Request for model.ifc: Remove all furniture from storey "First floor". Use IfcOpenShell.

First a look at what the model holds.

```python
import ifcopenshell
import ifcopenshell.util.element

model = ifcopenshell.open("model.ifc")
print(model.schema)
storey = next(s for s in model.by_type("IfcBuildingStorey") if s.Name == "First floor")
furniture = [e for e in ifcopenshell.util.element.get_decomposition(storey) if e.is_a("IfcFurnishingElement")]
seen = {}
for e in furniture:
    element_type = ifcopenshell.util.element.get_type(e)
    name = element_type.Name if element_type not in (None, e) else None
    seen[name] = seen.get(name, 0) + 1
for name, count in sorted(seen.items(), key=str):
    print(count, "x", name)
```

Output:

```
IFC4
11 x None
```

```python
import ifcopenshell
import ifcopenshell.api.root
import ifcopenshell.util.element

model = ifcopenshell.open("model.ifc")

storey = next(s for s in model.by_type("IfcBuildingStorey") if s.Name == "First floor")
furniture = [e for e in ifcopenshell.util.element.get_decomposition(storey) if e.is_a("IfcFurnishingElement")]

for e in furniture:
    ifcopenshell.api.root.remove_product(model, product=e)
print(len(furniture), "removed")

model.write("model_v2.ifc")
```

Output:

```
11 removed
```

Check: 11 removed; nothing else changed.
